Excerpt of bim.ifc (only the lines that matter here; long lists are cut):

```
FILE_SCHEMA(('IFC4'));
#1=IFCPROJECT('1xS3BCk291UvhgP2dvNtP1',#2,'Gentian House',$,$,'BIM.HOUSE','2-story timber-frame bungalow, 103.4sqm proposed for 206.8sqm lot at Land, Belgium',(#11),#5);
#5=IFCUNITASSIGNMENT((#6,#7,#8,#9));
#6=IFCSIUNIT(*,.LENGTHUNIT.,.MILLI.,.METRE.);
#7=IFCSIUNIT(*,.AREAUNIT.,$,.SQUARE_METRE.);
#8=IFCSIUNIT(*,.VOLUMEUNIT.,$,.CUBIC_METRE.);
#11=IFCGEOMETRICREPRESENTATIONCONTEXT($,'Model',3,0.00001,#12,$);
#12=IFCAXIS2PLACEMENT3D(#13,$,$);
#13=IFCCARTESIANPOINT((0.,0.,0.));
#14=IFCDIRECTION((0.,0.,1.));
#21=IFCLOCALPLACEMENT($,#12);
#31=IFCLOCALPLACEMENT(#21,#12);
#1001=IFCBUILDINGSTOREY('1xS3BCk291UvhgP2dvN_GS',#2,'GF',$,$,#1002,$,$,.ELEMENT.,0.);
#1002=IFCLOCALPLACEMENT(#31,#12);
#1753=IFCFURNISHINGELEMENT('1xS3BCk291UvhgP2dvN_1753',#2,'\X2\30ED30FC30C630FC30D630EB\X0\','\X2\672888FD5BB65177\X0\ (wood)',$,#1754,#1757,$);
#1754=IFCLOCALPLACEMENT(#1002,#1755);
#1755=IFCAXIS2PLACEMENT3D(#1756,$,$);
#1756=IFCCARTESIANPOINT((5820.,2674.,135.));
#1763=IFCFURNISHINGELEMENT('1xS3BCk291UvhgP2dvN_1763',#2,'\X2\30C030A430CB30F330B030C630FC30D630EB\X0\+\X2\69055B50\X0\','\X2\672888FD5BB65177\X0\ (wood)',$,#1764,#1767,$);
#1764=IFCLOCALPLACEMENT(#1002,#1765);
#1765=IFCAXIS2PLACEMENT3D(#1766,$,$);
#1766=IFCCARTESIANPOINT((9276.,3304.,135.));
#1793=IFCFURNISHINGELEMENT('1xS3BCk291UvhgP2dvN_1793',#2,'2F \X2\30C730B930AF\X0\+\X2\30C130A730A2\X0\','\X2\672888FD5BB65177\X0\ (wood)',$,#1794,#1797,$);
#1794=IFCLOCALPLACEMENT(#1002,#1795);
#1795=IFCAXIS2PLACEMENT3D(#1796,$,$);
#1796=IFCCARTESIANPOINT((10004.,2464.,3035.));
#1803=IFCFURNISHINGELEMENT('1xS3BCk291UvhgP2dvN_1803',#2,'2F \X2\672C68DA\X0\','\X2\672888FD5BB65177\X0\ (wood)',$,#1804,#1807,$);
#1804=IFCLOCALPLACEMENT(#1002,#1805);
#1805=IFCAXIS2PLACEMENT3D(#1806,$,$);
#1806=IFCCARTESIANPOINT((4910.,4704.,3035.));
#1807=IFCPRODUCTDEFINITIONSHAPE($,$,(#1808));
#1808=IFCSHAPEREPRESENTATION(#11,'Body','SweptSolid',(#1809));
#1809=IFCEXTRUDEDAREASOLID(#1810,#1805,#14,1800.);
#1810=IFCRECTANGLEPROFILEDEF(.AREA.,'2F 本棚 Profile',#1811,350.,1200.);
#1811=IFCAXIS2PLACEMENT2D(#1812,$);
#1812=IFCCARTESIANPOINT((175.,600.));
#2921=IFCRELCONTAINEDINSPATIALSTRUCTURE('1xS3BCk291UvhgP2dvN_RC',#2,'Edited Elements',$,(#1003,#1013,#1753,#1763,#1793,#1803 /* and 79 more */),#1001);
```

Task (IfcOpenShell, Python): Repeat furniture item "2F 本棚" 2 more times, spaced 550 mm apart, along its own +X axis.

```python
import ifcopenshell
import ifcopenshell.api.geometry
import ifcopenshell.api.root
import ifcopenshell.util.element
import ifcopenshell.util.placement

model = ifcopenshell.open("bim.ifc")


def reuse_history(source, copy):
    """copy_class also copies each property set's owner history, people and application; keep the originals."""
    for rel in copy.IsDefinedBy:
        if rel.is_a("IfcRelDefinesByProperties") and (history := rel.RelatingPropertyDefinition.OwnerHistory):
            rel.RelatingPropertyDefinition.OwnerHistory = source.OwnerHistory
            ifcopenshell.util.element.remove_deep2(model, history)


source = model.by_id(1803)
base = ifcopenshell.util.placement.get_local_placement(source.ObjectPlacement)
step = base[:3, 0] * 550.0

for i in range(1, 3):
    copy = ifcopenshell.api.root.copy_class(model, product=source)
    copy.Representation = ifcopenshell.util.element.copy_deep(
        model, source.Representation, exclude=["IfcGeometricRepresentationContext", "IfcRepresentationMap"]
    )
    reuse_history(source, copy)
    matrix = base.copy()
    matrix[:3, 3] += i * step
    print("added at", matrix[:3, 3].round(3) + 0.0)
    ifcopenshell.api.geometry.edit_object_placement(model, product=copy, matrix=matrix, is_si=False)

model.write("bim_updated.ifc")
```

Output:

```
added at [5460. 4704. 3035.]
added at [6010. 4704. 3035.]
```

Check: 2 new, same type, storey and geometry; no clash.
